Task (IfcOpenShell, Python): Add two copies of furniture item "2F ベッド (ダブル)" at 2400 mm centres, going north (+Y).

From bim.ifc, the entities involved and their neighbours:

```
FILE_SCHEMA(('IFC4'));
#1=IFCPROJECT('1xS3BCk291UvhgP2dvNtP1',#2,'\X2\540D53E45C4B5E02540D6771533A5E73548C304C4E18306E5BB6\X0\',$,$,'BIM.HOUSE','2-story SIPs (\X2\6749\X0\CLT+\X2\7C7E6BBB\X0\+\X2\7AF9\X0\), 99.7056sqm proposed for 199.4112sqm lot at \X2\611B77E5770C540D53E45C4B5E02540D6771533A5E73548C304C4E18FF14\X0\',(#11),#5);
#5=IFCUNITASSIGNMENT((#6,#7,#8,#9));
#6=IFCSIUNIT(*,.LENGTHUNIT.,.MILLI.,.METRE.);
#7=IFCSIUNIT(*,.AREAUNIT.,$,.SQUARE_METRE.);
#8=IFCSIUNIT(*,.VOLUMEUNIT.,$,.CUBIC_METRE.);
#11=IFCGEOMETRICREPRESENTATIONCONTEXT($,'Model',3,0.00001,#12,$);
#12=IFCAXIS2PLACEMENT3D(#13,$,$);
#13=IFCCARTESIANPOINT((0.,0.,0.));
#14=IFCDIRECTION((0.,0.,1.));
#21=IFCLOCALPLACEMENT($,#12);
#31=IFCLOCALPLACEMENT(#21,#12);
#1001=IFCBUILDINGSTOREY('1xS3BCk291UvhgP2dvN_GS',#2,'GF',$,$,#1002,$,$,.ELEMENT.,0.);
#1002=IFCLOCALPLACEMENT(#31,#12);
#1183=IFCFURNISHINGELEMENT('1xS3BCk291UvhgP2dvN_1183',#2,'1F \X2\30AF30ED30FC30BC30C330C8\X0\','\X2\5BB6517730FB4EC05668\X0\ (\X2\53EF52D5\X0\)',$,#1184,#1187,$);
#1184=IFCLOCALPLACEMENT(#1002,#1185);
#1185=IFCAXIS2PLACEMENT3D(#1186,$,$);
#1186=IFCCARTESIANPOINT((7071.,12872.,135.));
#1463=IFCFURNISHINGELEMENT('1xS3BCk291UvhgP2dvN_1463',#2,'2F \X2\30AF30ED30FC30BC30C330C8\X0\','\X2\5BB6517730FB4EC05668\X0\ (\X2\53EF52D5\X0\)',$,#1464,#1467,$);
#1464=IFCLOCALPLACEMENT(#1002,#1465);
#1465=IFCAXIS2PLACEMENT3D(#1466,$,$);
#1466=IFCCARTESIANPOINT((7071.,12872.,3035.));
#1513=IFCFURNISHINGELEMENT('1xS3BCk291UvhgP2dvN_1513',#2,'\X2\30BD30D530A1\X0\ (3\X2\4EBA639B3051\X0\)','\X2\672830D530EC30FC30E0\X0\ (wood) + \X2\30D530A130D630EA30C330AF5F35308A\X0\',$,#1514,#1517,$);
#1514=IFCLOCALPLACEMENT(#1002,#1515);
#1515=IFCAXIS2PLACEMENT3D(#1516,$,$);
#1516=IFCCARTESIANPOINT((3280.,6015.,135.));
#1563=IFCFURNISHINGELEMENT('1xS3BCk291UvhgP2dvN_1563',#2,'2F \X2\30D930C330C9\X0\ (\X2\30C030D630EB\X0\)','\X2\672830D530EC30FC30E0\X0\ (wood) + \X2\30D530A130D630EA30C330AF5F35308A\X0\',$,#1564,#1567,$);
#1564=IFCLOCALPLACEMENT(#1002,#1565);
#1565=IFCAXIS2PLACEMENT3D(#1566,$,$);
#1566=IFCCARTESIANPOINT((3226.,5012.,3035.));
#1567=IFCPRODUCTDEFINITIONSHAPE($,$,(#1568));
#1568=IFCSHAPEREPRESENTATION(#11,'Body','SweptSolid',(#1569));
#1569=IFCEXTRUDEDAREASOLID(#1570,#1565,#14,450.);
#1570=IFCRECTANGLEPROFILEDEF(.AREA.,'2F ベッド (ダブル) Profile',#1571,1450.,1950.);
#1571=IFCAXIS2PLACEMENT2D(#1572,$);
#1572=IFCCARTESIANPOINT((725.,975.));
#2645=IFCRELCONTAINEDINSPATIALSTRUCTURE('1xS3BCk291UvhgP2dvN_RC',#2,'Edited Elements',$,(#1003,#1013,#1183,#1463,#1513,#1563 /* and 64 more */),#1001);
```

```python
import numpy as np
import ifcopenshell
import ifcopenshell.api.geometry
import ifcopenshell.api.root
import ifcopenshell.util.element
import ifcopenshell.util.placement

model = ifcopenshell.open("bim.ifc")


def reuse_history(source, copy):
    """copy_class also copies each property set's owner history, people and application; keep the originals."""
    for rel in copy.IsDefinedBy:
        if rel.is_a("IfcRelDefinesByProperties") and (history := rel.RelatingPropertyDefinition.OwnerHistory):
            rel.RelatingPropertyDefinition.OwnerHistory = source.OwnerHistory
            ifcopenshell.util.element.remove_deep2(model, history)


source = model.by_id(1563)
base = ifcopenshell.util.placement.get_local_placement(source.ObjectPlacement)
step = np.array([0.0, 1.0, 0.0]) * 2400.0

for i in range(1, 3):
    copy = ifcopenshell.api.root.copy_class(model, product=source)
    copy.Representation = ifcopenshell.util.element.copy_deep(
        model, source.Representation, exclude=["IfcGeometricRepresentationContext", "IfcRepresentationMap"]
    )
    reuse_history(source, copy)
    matrix = base.copy()
    matrix[:3, 3] += i * step
    print("added at", matrix[:3, 3].round(3) + 0.0)
    ifcopenshell.api.geometry.edit_object_placement(model, product=copy, matrix=matrix, is_si=False)

model.write("bim_updated.ifc")
```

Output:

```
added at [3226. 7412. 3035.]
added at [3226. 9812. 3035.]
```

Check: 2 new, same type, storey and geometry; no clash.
